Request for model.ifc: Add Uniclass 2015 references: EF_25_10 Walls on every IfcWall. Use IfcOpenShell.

First a look at what the model holds.

```python
import ifcopenshell

model = ifcopenshell.open("model.ifc")
print(model.schema)
print("classifications:", [c.Name for c in model.by_type("IfcClassification")])
for ifc_class in ("IfcDoor", "IfcRoof", "IfcStair", "IfcWall", "IfcWindow"):
    print(ifc_class, len(model.by_type(ifc_class)))
```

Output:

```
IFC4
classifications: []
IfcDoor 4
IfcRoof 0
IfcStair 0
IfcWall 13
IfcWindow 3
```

```python
import ifcopenshell
import ifcopenshell.api.classification

model = ifcopenshell.open("model.ifc")

system = ifcopenshell.api.classification.add_classification(model, classification="Uniclass 2015")

codes = {
    "IfcWall": ("EF_25_10", "Walls"),
}
for ifc_class, (code, name) in codes.items():
    products = model.by_type(ifc_class)
    ifcopenshell.api.classification.add_reference(
        model, products=products, classification=system, identification=code, name=name
    )
    print(code, len(products))

model.write("model_rev.ifc")
```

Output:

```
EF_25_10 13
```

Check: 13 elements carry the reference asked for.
